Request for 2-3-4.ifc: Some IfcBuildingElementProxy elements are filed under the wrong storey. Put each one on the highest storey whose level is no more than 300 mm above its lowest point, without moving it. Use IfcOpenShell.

First a look at what the model holds.

```python
import ifcopenshell
import ifcopenshell.util.element
import ifcopenshell.util.placement

model = ifcopenshell.open("2-3-4.ifc")
print(model.schema)
for storey in model.by_type("IfcBuildingStorey"):
    level = ifcopenshell.util.placement.get_storey_elevation(storey)
    count = sum(e.is_a("IfcBuildingElementProxy") for e in ifcopenshell.util.element.get_contained(storey))
    print(storey.id(), storey.Name, round(level, 3), count, sep=" | ")
```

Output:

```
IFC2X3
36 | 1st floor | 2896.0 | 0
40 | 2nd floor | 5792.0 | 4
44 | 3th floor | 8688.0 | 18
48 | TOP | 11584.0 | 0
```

```python
import ifcopenshell
import ifcopenshell.api.spatial
import ifcopenshell.geom
import ifcopenshell.util.element
import ifcopenshell.util.placement
import ifcopenshell.util.shape
import ifcopenshell.util.unit

model = ifcopenshell.open("2-3-4.ifc")
unit_scale = ifcopenshell.util.unit.calculate_unit_scale(model)
settings = ifcopenshell.geom.settings()

levels = sorted(
    ((ifcopenshell.util.placement.get_storey_elevation(s) * unit_scale, s) for s in model.by_type("IfcBuildingStorey")),
    key=lambda pair: pair[0],
)

for e in model.by_type("IfcBuildingElementProxy"):
    current = e.ContainedInStructure[0].RelatingStructure if e.ContainedInStructure else None
    if current is None or not current.is_a("IfcBuildingStorey"):
        continue
    shape = ifcopenshell.geom.create_shape(settings, e)
    bottom = ifcopenshell.util.shape.get_shape_bottom_elevation(shape, shape.geometry)
    below = [s for level, s in levels if level <= bottom + 0.3]
    storey = below[-1] if below else levels[0][1]
    if storey != current:
        # assign_container keeps the world position.
        ifcopenshell.api.spatial.assign_container(model, products=[e], relating_structure=storey)
        print(e.id(), current.Name, "->", storey.Name)

model.write("2-3-4_v2.ifc")
```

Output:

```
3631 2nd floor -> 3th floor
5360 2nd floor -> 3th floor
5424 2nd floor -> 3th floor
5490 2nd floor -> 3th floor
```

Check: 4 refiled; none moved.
